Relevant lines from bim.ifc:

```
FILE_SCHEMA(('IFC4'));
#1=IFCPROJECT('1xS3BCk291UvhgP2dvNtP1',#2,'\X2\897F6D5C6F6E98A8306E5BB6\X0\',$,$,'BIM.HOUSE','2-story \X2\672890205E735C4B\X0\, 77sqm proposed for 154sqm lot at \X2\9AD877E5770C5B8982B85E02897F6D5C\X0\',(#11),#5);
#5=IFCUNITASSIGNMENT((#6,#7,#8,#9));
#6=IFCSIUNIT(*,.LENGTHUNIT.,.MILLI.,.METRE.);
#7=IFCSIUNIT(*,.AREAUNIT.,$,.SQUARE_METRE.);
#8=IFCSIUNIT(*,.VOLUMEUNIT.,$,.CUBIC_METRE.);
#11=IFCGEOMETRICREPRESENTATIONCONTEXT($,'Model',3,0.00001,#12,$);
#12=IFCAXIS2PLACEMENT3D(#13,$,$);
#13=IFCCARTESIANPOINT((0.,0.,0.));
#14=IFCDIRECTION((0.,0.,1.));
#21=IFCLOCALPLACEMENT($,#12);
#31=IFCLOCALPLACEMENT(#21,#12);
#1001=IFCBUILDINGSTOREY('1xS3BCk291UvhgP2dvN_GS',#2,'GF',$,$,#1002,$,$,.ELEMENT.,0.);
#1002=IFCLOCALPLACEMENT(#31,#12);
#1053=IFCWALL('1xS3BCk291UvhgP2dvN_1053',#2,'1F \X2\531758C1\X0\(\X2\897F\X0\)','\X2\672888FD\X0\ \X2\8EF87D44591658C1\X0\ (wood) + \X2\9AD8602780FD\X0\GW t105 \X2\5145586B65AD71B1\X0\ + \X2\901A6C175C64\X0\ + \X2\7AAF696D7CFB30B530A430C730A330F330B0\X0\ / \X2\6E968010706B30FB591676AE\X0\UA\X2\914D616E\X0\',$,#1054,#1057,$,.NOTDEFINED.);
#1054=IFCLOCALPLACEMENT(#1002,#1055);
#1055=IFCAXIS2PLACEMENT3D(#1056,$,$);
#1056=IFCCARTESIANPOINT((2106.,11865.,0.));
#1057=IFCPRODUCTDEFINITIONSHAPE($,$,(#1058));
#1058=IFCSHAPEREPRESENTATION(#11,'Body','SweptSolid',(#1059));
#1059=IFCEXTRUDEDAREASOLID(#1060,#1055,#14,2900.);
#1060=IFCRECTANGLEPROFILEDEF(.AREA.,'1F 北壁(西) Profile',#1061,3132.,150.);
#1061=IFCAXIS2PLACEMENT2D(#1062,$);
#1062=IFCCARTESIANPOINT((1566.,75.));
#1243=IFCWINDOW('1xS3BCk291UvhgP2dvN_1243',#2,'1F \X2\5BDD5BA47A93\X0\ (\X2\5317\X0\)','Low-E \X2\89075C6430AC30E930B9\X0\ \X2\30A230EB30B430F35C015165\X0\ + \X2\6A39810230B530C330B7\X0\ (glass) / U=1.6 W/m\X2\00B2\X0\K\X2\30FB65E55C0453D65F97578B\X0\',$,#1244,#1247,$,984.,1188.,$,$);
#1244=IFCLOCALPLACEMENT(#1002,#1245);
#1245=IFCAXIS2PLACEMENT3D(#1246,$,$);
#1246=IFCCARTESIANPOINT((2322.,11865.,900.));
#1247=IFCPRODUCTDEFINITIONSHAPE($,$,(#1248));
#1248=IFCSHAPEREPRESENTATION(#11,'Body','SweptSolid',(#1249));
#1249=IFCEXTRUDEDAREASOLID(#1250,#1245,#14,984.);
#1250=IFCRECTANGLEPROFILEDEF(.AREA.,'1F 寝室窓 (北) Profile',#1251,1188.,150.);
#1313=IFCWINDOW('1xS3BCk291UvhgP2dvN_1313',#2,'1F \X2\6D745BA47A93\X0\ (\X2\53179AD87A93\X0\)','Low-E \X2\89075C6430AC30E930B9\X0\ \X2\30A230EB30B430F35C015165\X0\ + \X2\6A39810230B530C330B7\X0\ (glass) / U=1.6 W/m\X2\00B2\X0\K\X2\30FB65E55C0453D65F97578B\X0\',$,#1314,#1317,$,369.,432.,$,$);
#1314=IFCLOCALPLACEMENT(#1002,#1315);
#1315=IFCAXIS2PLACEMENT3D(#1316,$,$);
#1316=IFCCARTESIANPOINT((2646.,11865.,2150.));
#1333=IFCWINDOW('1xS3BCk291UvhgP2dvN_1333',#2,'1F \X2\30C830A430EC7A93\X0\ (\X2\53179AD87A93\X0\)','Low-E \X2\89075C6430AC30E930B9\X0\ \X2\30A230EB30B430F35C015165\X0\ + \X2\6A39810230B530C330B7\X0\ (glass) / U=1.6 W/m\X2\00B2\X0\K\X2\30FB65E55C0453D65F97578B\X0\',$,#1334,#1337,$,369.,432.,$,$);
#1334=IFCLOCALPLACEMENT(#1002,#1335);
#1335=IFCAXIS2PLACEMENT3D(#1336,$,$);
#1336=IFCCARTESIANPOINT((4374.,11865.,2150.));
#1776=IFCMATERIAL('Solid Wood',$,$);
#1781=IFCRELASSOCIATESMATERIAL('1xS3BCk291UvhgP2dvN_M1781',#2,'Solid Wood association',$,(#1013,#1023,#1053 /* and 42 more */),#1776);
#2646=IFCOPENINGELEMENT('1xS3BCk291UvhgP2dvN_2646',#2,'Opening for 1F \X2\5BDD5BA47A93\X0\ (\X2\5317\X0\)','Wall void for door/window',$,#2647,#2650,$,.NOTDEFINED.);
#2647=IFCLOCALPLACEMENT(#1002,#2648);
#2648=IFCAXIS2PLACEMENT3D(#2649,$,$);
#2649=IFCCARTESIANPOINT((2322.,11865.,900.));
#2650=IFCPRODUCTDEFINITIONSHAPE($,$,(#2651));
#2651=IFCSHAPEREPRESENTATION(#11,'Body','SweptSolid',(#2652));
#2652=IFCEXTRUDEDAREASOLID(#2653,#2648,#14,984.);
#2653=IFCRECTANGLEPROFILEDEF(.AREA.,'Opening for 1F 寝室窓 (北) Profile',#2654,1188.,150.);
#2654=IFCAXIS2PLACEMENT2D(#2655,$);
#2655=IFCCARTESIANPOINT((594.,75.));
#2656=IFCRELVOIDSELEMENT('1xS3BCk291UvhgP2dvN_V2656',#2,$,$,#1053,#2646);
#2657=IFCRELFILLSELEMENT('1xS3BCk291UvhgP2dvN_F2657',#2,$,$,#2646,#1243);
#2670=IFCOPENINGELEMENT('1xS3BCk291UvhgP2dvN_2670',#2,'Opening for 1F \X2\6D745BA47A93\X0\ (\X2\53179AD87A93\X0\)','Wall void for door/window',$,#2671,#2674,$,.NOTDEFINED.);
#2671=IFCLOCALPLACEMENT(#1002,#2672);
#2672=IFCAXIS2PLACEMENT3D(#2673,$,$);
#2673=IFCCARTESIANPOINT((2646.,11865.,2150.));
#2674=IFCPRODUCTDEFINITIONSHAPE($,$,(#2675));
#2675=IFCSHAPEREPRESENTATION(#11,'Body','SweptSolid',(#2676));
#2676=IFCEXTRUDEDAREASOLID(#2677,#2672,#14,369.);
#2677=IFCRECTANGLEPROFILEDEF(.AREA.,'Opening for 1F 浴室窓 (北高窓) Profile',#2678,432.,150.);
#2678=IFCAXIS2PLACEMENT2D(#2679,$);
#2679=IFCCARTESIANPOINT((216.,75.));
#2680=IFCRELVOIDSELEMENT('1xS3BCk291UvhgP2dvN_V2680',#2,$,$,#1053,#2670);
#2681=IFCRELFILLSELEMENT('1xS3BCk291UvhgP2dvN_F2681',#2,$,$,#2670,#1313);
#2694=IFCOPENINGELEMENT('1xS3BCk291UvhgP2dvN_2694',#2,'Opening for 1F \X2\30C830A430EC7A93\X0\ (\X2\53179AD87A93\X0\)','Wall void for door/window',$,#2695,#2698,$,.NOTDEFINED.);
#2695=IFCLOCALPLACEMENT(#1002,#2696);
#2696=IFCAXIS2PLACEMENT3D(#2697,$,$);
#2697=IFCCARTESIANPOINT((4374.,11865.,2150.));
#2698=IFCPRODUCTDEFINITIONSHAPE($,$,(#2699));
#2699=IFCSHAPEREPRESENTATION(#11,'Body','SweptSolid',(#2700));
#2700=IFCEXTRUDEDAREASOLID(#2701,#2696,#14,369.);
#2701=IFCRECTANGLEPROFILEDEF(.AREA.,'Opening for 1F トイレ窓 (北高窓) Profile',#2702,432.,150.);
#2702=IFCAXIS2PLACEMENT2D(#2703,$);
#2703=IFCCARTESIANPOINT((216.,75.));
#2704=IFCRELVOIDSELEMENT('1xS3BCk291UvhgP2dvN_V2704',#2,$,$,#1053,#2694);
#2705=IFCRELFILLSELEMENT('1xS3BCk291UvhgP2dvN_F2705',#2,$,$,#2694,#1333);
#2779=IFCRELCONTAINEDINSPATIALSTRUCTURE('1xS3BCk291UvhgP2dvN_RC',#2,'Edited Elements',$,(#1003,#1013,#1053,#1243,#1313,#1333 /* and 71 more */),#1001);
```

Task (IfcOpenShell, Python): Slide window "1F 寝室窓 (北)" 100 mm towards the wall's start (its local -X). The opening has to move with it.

```python
import ifcopenshell
import ifcopenshell.api.geometry
import ifcopenshell.util.placement
import ifcopenshell.util.unit

model = ifcopenshell.open("bim.ifc")
unit_scale = ifcopenshell.util.unit.calculate_unit_scale(model)

window = model.by_guid("1xS3BCk291UvhgP2dvN_1243")
opening = window.FillsVoids[0].RelatingOpeningElement
wall = opening.VoidsElements[0].RelatingBuildingElement

wall_matrix = ifcopenshell.util.placement.get_local_placement(wall.ObjectPlacement)
shift = wall_matrix[:3, 0] * -0.1 / unit_scale
before = ifcopenshell.util.placement.get_local_placement(window.ObjectPlacement)[:3, 3].copy()

# The window is not placed relative to its opening, so move both.
for product in (opening, window):
    matrix = ifcopenshell.util.placement.get_local_placement(product.ObjectPlacement)
    matrix[:3, 3] += shift
    ifcopenshell.api.geometry.edit_object_placement(model, product=product, matrix=matrix, is_si=False)

after = ifcopenshell.util.placement.get_local_placement(window.ObjectPlacement)[:3, 3]
print("window moved by", (after - before).round(3) + 0.0)

model.write("bim_rev.ifc")
```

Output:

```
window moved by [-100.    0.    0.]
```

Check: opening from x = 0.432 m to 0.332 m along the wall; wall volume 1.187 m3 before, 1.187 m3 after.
